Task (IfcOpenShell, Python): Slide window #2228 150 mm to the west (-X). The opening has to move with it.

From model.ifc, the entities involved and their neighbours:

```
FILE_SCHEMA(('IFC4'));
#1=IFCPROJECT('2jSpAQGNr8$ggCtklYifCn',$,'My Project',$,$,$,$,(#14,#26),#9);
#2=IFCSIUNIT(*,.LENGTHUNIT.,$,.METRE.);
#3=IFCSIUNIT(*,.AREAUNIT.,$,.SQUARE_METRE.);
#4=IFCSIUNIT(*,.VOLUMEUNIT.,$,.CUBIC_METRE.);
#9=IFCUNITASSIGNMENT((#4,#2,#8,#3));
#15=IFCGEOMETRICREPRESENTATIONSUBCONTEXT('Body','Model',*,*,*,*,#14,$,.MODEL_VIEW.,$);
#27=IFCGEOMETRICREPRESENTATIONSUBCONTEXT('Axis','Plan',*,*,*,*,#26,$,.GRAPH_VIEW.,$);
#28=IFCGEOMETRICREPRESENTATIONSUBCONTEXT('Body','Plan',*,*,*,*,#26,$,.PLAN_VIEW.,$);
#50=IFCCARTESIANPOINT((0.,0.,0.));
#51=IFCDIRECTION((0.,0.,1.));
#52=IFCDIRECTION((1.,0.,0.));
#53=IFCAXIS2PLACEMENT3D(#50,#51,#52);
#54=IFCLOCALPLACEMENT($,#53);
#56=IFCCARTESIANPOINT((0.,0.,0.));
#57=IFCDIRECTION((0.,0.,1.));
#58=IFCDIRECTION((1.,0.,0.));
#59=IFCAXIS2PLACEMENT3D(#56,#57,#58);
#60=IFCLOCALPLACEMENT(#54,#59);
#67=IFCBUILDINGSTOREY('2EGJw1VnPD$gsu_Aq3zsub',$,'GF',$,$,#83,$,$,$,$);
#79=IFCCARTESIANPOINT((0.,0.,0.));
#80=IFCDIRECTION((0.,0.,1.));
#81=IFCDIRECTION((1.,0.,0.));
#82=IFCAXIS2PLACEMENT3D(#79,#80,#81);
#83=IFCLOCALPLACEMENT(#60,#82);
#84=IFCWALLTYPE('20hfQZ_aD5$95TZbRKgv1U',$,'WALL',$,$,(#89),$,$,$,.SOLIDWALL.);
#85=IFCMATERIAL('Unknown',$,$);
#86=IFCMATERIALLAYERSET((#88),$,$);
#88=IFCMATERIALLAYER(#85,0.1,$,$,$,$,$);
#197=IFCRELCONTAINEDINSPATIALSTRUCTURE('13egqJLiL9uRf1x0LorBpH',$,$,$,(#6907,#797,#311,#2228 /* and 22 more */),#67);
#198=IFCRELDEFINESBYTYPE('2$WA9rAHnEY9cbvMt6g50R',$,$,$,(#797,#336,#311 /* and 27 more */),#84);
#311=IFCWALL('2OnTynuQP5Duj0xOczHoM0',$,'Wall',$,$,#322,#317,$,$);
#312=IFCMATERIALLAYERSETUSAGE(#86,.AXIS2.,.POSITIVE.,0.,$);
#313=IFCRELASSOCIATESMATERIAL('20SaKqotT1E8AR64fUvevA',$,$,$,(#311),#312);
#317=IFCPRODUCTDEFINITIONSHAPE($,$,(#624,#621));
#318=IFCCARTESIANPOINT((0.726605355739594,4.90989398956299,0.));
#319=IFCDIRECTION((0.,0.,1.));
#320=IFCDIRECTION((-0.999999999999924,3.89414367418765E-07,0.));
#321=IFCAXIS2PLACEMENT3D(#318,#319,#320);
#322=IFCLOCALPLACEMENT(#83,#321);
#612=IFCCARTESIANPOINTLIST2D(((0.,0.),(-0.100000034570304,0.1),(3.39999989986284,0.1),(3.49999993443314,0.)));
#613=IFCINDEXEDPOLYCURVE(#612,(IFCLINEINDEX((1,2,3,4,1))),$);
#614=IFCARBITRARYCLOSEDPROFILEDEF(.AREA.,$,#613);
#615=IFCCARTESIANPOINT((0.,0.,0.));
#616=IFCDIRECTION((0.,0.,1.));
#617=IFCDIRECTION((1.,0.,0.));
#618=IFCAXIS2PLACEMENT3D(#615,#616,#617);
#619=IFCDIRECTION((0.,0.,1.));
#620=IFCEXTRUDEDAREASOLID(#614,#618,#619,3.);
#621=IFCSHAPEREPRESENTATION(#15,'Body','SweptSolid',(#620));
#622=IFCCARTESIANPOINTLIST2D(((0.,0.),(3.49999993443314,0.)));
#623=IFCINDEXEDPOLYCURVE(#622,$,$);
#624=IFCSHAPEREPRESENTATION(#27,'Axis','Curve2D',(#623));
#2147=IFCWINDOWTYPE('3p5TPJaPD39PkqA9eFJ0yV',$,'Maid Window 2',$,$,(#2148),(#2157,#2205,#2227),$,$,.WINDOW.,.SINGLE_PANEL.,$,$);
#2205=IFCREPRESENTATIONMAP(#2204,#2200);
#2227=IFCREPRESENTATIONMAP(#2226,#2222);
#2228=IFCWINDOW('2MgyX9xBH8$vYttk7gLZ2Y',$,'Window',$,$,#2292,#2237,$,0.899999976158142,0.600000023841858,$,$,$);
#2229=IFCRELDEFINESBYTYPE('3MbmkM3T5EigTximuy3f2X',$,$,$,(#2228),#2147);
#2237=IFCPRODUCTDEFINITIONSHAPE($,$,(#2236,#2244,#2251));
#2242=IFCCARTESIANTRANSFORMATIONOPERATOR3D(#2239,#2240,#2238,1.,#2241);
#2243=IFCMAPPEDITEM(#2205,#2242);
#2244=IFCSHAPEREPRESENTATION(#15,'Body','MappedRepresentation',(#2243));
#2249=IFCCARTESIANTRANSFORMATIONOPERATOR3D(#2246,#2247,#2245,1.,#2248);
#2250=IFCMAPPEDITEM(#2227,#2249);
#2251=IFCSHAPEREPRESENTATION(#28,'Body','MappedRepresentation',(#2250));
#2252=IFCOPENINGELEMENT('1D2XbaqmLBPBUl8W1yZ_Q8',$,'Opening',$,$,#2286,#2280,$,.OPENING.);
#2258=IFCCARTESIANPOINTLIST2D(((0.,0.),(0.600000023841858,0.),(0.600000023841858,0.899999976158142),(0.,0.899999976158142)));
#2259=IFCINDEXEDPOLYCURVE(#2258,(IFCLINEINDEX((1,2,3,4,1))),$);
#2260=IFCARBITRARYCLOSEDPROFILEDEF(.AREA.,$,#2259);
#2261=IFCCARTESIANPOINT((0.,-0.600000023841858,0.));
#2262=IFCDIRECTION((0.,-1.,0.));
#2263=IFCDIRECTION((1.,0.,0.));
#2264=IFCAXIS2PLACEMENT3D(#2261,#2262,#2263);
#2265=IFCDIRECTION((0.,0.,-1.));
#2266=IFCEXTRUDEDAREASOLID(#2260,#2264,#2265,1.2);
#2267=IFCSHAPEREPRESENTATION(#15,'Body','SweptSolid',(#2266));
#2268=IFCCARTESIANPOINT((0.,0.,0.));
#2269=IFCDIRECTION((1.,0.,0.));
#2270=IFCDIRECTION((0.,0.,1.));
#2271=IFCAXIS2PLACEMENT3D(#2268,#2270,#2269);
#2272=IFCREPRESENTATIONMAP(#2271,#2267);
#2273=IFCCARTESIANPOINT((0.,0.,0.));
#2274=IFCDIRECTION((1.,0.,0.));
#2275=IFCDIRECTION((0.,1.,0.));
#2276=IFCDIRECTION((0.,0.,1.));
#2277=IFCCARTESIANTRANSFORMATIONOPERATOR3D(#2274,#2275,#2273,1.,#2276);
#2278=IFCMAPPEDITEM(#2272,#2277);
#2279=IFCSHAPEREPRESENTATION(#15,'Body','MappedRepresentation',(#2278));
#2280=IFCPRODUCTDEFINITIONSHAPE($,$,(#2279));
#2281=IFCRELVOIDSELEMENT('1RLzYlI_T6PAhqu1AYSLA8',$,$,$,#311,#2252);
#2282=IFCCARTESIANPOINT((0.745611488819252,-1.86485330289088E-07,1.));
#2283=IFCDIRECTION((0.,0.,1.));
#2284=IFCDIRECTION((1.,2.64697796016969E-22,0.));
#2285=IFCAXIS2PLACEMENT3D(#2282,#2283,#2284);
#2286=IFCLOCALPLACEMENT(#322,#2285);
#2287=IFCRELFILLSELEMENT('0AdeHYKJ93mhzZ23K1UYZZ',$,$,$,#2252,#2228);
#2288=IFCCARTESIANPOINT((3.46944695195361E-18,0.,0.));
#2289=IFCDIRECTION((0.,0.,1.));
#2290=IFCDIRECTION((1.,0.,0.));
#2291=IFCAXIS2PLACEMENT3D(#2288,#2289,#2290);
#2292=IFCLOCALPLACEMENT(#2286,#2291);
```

```python
import ifcopenshell
import ifcopenshell.api.geometry
import ifcopenshell.util.placement
import ifcopenshell.util.unit

model = ifcopenshell.open("model.ifc")
unit_scale = ifcopenshell.util.unit.calculate_unit_scale(model)

window = model.by_guid("2MgyX9xBH8$vYttk7gLZ2Y")
opening = window.FillsVoids[0].RelatingOpeningElement
wall = opening.VoidsElements[0].RelatingBuildingElement

wall_matrix = ifcopenshell.util.placement.get_local_placement(wall.ObjectPlacement)
shift = wall_matrix[:3, 0] * 0.15 / unit_scale
before = ifcopenshell.util.placement.get_local_placement(window.ObjectPlacement)[:3, 3].copy()

# The window is placed relative to its opening, so it follows when the opening moves.
matrix = ifcopenshell.util.placement.get_local_placement(opening.ObjectPlacement)
matrix[:3, 3] += shift
ifcopenshell.api.geometry.edit_object_placement(
    model, product=opening, matrix=matrix, is_si=False, should_transform_children=True
)

after = ifcopenshell.util.placement.get_local_placement(window.ObjectPlacement)[:3, 3]
print("window moved by", (after - before).round(3) + 0.0)

model.write("model_updated.ifc")
```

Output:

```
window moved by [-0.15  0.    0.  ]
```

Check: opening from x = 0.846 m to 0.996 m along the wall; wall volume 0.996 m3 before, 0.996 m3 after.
